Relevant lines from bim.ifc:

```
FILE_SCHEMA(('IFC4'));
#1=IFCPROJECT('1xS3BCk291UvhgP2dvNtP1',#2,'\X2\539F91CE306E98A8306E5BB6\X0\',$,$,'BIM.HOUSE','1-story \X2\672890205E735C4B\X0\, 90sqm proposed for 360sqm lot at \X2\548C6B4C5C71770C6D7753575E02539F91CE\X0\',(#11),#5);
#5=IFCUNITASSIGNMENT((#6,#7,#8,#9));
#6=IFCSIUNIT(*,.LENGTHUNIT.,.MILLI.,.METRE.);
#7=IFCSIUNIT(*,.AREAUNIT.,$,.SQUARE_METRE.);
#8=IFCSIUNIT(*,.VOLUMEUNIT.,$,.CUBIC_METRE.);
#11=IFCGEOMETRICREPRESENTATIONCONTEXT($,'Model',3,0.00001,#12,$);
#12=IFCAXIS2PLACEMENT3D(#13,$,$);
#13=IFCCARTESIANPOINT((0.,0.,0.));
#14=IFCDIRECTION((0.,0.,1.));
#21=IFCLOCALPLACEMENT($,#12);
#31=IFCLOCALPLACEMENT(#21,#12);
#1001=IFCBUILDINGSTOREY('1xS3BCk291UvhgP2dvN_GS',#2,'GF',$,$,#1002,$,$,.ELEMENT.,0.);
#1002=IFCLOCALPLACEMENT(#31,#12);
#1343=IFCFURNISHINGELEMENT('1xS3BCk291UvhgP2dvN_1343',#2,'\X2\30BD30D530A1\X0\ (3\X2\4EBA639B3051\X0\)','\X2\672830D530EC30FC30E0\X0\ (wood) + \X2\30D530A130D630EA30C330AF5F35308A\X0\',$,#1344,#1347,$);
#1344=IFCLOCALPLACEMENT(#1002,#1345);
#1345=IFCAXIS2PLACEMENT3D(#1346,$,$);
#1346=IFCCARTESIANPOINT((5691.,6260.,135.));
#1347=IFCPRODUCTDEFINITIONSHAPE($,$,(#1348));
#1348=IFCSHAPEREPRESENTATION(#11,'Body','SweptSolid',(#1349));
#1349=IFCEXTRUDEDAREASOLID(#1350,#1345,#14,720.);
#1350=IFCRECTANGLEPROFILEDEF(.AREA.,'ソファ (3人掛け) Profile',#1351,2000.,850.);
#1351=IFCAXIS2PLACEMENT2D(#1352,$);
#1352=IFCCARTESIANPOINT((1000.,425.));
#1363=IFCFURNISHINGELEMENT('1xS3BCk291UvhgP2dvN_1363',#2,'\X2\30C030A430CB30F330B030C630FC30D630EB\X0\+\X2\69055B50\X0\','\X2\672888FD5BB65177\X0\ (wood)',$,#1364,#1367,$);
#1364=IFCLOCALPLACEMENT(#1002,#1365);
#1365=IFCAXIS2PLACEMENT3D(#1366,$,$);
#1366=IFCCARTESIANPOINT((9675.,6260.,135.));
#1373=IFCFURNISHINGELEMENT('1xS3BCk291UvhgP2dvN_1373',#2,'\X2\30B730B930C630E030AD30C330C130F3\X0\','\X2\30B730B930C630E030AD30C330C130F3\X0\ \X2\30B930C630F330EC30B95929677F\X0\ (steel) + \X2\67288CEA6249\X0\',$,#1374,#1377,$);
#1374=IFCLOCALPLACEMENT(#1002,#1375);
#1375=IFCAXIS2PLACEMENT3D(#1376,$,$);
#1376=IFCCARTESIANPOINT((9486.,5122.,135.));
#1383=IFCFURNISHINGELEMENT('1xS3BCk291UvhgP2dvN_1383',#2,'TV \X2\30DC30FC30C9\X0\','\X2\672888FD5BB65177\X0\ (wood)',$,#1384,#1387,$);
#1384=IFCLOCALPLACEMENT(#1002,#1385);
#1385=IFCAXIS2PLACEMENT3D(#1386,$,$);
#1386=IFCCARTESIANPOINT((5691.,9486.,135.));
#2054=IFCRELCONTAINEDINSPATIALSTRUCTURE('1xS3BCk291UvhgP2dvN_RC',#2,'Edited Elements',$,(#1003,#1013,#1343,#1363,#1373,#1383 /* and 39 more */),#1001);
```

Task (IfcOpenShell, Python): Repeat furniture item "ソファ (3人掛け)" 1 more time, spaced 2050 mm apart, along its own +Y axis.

```python
import ifcopenshell
import ifcopenshell.api.geometry
import ifcopenshell.api.root
import ifcopenshell.util.element
import ifcopenshell.util.placement
import ifcopenshell.util.unit

model = ifcopenshell.open("bim.ifc")
unit_scale = ifcopenshell.util.unit.calculate_unit_scale(model)


def reuse_history(source, copy):
    """copy_class also copies each property set's owner history, people and application; keep the originals."""
    for rel in copy.IsDefinedBy:
        if rel.is_a("IfcRelDefinesByProperties") and (history := rel.RelatingPropertyDefinition.OwnerHistory):
            rel.RelatingPropertyDefinition.OwnerHistory = source.OwnerHistory
            ifcopenshell.util.element.remove_deep2(model, history)


source = model.by_guid("1xS3BCk291UvhgP2dvN_1343")
base = ifcopenshell.util.placement.get_local_placement(source.ObjectPlacement)
step = base[:3, 1] * 2.05 / unit_scale

for i in range(1, 2):
    copy = ifcopenshell.api.root.copy_class(model, product=source)
    copy.Representation = ifcopenshell.util.element.copy_deep(
        model, source.Representation, exclude=["IfcGeometricRepresentationContext", "IfcRepresentationMap"]
    )
    reuse_history(source, copy)
    matrix = base.copy()
    matrix[:3, 3] += i * step
    print("added at", matrix[:3, 3].round(3) + 0.0)
    ifcopenshell.api.geometry.edit_object_placement(model, product=copy, matrix=matrix, is_si=False)

model.write("bim_updated.ifc")
```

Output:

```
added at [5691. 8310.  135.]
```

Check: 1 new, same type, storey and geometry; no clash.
